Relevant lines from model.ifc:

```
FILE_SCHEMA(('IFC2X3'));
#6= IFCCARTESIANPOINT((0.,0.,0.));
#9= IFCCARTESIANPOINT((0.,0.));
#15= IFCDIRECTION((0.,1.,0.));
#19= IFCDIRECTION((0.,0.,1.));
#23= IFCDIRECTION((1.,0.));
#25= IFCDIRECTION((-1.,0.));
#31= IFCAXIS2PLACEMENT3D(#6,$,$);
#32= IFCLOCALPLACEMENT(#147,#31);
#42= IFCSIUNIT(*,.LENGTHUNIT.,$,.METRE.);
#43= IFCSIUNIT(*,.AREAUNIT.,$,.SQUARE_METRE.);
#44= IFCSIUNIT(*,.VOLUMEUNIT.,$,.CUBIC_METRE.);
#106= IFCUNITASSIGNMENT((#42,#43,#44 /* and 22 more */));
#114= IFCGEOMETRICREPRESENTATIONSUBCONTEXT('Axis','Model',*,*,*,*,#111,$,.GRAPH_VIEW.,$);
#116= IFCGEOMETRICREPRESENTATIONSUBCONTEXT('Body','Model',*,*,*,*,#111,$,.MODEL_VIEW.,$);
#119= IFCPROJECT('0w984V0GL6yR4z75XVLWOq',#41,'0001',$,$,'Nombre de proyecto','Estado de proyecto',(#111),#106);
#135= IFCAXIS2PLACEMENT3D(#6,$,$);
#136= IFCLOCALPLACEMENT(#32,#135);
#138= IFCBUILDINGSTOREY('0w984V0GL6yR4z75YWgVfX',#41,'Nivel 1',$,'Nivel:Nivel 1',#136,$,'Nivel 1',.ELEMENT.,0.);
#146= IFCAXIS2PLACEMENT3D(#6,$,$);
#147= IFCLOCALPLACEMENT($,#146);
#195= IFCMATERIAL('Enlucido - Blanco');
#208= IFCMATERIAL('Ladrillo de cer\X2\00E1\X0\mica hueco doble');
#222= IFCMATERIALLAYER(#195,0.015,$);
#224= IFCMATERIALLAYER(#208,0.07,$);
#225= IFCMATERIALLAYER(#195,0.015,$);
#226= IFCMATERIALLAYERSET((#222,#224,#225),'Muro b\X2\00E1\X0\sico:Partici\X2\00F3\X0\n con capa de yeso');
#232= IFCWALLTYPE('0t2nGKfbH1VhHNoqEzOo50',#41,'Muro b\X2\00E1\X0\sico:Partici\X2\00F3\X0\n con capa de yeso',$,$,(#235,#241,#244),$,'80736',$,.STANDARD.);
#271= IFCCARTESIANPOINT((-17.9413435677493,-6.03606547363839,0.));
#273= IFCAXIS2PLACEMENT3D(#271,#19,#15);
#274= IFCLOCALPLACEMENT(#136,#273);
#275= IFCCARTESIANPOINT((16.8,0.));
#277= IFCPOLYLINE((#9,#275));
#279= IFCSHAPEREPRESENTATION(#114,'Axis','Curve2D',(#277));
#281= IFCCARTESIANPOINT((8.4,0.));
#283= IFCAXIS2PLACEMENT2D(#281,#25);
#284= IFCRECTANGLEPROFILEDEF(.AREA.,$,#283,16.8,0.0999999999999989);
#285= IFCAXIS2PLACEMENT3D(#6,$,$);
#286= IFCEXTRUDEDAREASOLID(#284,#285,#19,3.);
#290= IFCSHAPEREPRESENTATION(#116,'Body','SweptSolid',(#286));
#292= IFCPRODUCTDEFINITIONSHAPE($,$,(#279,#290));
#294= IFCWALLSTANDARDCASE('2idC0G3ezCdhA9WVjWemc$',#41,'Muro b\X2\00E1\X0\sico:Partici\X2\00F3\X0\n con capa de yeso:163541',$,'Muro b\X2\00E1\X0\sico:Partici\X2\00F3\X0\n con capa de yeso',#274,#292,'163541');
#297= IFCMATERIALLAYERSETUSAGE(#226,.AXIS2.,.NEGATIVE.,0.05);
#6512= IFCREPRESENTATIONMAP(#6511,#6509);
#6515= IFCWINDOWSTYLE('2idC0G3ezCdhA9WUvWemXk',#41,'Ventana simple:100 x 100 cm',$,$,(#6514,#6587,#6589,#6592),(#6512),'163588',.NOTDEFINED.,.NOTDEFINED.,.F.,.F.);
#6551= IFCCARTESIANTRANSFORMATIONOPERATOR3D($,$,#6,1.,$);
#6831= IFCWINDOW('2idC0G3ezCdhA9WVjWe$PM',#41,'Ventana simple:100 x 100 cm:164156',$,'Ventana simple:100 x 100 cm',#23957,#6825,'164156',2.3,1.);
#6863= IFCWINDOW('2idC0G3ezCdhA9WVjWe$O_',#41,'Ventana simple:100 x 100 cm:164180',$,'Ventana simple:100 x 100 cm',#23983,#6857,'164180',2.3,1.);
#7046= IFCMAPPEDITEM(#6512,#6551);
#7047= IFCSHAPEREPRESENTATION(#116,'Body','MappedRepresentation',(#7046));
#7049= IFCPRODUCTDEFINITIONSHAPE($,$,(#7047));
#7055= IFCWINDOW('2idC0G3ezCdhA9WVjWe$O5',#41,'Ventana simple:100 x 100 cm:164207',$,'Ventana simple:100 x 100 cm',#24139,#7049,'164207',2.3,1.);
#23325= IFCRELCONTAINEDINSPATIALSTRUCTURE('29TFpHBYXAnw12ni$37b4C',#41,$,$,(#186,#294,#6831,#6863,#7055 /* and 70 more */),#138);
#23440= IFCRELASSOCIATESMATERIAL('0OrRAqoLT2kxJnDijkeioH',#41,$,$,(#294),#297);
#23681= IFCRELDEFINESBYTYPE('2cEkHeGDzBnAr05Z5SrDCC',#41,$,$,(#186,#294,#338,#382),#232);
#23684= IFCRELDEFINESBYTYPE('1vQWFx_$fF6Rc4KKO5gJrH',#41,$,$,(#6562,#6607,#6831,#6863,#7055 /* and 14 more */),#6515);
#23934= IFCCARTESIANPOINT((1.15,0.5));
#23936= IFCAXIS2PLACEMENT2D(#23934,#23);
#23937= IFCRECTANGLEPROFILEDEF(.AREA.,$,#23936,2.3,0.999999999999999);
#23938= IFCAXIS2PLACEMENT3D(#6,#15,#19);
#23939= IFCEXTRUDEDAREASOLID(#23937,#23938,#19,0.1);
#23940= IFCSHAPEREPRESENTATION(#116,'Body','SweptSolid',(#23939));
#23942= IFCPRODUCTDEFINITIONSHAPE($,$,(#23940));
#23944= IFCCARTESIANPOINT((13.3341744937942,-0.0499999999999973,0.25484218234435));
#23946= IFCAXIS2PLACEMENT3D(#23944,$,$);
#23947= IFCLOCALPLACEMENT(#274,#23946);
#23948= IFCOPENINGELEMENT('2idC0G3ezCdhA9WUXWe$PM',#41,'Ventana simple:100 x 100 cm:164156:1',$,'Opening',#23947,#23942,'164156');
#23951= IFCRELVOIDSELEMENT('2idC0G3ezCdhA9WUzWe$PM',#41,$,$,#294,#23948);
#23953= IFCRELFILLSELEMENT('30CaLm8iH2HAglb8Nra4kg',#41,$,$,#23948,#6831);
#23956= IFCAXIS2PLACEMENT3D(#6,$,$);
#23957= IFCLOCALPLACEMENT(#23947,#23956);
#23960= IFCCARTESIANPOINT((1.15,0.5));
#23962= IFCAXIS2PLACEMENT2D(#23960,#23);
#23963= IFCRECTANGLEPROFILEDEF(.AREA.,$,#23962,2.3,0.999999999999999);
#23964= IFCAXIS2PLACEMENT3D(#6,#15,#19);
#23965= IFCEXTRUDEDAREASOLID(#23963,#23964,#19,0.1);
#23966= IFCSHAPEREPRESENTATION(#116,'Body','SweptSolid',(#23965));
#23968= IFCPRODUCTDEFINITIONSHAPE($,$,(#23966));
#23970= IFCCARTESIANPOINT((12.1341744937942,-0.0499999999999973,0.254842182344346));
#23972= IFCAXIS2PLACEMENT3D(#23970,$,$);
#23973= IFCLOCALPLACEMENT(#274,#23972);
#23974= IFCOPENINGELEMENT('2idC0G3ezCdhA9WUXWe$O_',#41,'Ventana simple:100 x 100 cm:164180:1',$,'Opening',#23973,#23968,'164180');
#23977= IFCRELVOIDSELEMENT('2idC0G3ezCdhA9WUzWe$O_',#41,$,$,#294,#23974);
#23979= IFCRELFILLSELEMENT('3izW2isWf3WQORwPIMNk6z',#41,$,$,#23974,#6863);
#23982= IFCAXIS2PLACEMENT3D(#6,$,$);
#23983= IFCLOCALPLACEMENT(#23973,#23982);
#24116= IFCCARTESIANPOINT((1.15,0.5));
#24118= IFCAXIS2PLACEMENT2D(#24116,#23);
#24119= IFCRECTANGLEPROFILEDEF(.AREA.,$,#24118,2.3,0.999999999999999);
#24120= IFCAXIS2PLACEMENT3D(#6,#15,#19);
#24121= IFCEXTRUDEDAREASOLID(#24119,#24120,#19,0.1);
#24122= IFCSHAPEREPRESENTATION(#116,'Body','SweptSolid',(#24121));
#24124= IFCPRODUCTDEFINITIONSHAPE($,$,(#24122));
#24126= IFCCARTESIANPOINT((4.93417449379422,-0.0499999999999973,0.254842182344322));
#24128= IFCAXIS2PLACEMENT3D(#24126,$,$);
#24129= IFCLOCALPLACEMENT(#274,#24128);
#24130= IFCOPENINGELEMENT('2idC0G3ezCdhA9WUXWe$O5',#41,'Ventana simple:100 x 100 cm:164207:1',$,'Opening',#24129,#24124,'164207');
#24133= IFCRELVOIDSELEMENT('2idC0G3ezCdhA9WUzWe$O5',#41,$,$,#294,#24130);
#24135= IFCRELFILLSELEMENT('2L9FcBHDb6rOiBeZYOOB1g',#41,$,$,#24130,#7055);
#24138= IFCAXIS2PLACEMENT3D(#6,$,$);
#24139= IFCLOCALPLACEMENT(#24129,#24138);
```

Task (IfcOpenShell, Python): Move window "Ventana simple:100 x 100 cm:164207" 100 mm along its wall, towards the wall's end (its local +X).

```python
import ifcopenshell
import ifcopenshell.api.geometry
import ifcopenshell.util.placement
import ifcopenshell.util.unit

model = ifcopenshell.open("model.ifc")
unit_scale = ifcopenshell.util.unit.calculate_unit_scale(model)

window = model.by_id(7055)
opening = window.FillsVoids[0].RelatingOpeningElement
wall = opening.VoidsElements[0].RelatingBuildingElement

wall_matrix = ifcopenshell.util.placement.get_local_placement(wall.ObjectPlacement)
shift = wall_matrix[:3, 0] * 0.1 / unit_scale
before = ifcopenshell.util.placement.get_local_placement(window.ObjectPlacement)[:3, 3].copy()

# The window is placed relative to its opening, so it follows when the opening moves.
matrix = ifcopenshell.util.placement.get_local_placement(opening.ObjectPlacement)
matrix[:3, 3] += shift
ifcopenshell.api.geometry.edit_object_placement(
    model, product=opening, matrix=matrix, is_si=False, should_transform_children=True
)

after = ifcopenshell.util.placement.get_local_placement(window.ObjectPlacement)[:3, 3]
print("window moved by", (after - before).round(3) + 0.0)

model.write("model-out.ifc")
```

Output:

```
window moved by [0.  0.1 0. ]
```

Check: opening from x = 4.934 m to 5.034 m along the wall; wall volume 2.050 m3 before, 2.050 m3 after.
